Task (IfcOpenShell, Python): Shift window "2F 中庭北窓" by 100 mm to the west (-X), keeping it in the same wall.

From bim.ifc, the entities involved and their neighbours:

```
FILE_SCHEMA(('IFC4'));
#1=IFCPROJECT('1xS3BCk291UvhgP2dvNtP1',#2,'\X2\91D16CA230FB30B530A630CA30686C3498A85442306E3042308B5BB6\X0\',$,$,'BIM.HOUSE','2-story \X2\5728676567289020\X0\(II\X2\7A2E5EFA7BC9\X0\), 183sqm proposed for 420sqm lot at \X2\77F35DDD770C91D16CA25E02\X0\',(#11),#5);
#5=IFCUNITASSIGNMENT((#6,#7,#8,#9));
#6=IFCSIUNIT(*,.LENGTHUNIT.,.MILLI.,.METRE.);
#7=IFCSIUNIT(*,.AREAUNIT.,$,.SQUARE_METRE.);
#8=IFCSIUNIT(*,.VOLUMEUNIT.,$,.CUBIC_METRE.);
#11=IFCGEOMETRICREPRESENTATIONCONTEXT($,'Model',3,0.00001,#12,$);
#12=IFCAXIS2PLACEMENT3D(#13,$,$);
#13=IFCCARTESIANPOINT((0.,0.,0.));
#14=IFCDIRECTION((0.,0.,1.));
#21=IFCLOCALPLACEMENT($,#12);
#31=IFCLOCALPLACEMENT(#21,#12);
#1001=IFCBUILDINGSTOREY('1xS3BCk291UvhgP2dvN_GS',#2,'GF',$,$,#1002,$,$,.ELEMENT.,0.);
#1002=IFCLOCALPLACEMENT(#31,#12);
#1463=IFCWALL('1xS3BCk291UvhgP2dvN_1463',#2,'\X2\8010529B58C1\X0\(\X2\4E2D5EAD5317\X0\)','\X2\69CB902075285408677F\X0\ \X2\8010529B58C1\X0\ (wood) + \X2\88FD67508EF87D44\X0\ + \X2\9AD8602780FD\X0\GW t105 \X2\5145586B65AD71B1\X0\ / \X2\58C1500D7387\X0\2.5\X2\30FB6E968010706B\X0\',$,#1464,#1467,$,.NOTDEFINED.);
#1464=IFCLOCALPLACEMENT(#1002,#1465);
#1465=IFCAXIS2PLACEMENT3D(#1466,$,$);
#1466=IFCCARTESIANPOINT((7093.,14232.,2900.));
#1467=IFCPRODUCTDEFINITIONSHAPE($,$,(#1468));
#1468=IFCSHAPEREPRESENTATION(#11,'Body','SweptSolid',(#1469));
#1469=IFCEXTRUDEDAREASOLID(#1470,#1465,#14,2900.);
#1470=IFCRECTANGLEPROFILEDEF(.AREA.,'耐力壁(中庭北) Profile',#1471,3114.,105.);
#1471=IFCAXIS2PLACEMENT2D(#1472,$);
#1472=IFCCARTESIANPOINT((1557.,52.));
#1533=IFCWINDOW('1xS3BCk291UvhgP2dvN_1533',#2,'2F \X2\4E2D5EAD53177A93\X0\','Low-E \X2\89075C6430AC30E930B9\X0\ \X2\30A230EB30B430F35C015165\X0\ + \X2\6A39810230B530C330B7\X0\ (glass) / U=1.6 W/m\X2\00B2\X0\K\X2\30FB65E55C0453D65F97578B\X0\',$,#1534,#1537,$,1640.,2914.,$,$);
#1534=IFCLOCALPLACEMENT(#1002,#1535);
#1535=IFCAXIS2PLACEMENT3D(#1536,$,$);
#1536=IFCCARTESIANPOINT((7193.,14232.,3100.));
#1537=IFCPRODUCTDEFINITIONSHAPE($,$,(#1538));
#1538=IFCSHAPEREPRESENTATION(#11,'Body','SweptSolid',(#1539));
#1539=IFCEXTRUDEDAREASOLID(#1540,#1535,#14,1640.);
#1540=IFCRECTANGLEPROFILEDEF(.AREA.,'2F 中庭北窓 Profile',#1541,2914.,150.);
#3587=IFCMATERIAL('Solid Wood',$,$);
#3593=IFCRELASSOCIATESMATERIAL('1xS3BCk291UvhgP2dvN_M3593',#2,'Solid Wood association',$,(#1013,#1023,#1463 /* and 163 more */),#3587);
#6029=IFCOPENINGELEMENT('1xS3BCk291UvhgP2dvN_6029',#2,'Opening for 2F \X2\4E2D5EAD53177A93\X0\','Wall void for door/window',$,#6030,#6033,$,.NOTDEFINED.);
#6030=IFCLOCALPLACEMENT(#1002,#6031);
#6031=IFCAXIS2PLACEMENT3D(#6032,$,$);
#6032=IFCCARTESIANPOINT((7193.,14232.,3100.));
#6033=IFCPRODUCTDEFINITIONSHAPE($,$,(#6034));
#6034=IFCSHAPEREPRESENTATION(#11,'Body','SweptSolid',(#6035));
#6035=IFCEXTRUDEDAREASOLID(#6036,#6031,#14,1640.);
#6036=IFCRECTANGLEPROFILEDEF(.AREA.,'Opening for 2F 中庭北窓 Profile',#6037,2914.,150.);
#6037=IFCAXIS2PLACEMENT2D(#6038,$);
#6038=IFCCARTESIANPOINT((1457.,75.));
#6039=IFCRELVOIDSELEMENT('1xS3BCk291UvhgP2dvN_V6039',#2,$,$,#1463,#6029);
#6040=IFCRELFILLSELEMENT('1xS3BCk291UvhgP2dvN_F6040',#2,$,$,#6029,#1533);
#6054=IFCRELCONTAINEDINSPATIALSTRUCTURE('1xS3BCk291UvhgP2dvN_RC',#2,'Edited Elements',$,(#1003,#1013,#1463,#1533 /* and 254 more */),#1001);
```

```python
import ifcopenshell
import ifcopenshell.api.geometry
import ifcopenshell.util.placement
import ifcopenshell.util.unit

model = ifcopenshell.open("bim.ifc")
unit_scale = ifcopenshell.util.unit.calculate_unit_scale(model)

window = model.by_guid("1xS3BCk291UvhgP2dvN_1533")
opening = window.FillsVoids[0].RelatingOpeningElement
wall = opening.VoidsElements[0].RelatingBuildingElement

wall_matrix = ifcopenshell.util.placement.get_local_placement(wall.ObjectPlacement)
shift = wall_matrix[:3, 0] * -0.1 / unit_scale
before = ifcopenshell.util.placement.get_local_placement(window.ObjectPlacement)[:3, 3].copy()

# The window is not placed relative to its opening, so move both.
for product in (opening, window):
    matrix = ifcopenshell.util.placement.get_local_placement(product.ObjectPlacement)
    matrix[:3, 3] += shift
    ifcopenshell.api.geometry.edit_object_placement(model, product=product, matrix=matrix, is_si=False)

after = ifcopenshell.util.placement.get_local_placement(window.ObjectPlacement)[:3, 3]
print("window moved by", (after - before).round(3) + 0.0)

model.write("bim_rev.ifc")
```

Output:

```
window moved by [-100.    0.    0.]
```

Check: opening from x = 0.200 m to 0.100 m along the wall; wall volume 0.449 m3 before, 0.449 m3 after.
